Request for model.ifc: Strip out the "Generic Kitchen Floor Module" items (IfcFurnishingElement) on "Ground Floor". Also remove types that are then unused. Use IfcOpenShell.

First a look at what the model holds.

```python
import ifcopenshell
import ifcopenshell.util.element

model = ifcopenshell.open("model.ifc")
print(model.schema)
storey = next(s for s in model.by_type("IfcBuildingStorey") if s.Name == "Ground Floor")
furniture = [e for e in ifcopenshell.util.element.get_decomposition(storey) if e.is_a("IfcFurnishingElement")]
seen = {}
for e in furniture:
    element_type = ifcopenshell.util.element.get_type(e)
    name = element_type.Name if element_type not in (None, e) else None
    seen[name] = seen.get(name, 0) + 1
for name, count in sorted(seen.items(), key=str):
    print(count, "x", name)
```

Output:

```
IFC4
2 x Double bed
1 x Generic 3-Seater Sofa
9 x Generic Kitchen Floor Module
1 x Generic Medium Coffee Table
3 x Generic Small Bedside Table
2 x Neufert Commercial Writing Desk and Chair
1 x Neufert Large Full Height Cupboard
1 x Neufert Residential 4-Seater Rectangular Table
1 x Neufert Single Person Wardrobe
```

```python
import ifcopenshell
import ifcopenshell.api.root
import ifcopenshell.util.element

model = ifcopenshell.open("model.ifc")

storey = next(s for s in model.by_type("IfcBuildingStorey") if s.Name == "Ground Floor")
furniture = [e for e in ifcopenshell.util.element.get_decomposition(storey) if e.is_a("IfcFurnishingElement")]
targets = [e for e in furniture if (t := ifcopenshell.util.element.get_type(e)) not in (None, e) and t.Name == "Generic Kitchen Floor Module"]
types = {ifcopenshell.util.element.get_type(e) for e in targets} - {None, *targets}

for e in targets:
    ifcopenshell.api.root.remove_product(model, product=e)
print(len(targets), "removed")

unused = [t for t in types if not ifcopenshell.util.element.get_types(t)]
for t in unused:
    ifcopenshell.api.root.remove_product(model, product=t)
print(len(unused), "unused types removed")

model.write("model_v2.ifc")
```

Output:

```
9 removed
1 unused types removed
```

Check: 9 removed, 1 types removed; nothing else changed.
